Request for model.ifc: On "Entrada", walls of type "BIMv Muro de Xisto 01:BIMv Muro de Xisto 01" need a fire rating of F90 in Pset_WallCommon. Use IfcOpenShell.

First a look at what the model holds.

```python
import ifcopenshell
import ifcopenshell.util.element

model = ifcopenshell.open("model.ifc")
print(model.schema)
storey = next(s for s in model.by_type("IfcBuildingStorey") if s.Name == "Entrada")
walls = [e for e in ifcopenshell.util.element.get_decomposition(storey) if e.is_a("IfcWall")]
seen = {}
for e in walls:
    element_type = ifcopenshell.util.element.get_type(e)
    key = (element_type.Name if element_type != e and element_type else None, ifcopenshell.util.element.get_pset(e, "Pset_WallCommon", "FireRating"))
    seen[key] = seen.get(key, 0) + 1
for (name, value), count in sorted(seen.items(), key=str):
    print(count, "x", name, "|", value)
```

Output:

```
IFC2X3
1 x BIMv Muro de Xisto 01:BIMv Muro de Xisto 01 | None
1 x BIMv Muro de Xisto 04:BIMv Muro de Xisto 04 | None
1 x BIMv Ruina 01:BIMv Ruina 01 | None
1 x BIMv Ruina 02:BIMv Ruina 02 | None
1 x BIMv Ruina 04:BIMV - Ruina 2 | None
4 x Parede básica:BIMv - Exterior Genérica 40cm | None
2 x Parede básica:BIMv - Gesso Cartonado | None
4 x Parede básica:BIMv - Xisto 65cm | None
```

```python
import ifcopenshell
import ifcopenshell.api.pset
import ifcopenshell.util.element

model = ifcopenshell.open("model.ifc")

storey = next(s for s in model.by_type("IfcBuildingStorey") if s.Name == "Entrada")
walls = [e for e in ifcopenshell.util.element.get_decomposition(storey) if e.is_a("IfcWall")]

count = 0
for e in walls:
    element_type = ifcopenshell.util.element.get_type(e)
    if element_type in (None, e) or element_type.Name != "BIMv Muro de Xisto 01:BIMv Muro de Xisto 01":
        continue
    # add_pset returns the element's existing set when there is one.
    pset = ifcopenshell.api.pset.add_pset(model, product=e, name="Pset_WallCommon")
    ifcopenshell.api.pset.edit_pset(model, pset=pset, properties={"FireRating": "F90"})
    count += 1

print(count, "walls updated")

model.write("model_rev.ifc")
```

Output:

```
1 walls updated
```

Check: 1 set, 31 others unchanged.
